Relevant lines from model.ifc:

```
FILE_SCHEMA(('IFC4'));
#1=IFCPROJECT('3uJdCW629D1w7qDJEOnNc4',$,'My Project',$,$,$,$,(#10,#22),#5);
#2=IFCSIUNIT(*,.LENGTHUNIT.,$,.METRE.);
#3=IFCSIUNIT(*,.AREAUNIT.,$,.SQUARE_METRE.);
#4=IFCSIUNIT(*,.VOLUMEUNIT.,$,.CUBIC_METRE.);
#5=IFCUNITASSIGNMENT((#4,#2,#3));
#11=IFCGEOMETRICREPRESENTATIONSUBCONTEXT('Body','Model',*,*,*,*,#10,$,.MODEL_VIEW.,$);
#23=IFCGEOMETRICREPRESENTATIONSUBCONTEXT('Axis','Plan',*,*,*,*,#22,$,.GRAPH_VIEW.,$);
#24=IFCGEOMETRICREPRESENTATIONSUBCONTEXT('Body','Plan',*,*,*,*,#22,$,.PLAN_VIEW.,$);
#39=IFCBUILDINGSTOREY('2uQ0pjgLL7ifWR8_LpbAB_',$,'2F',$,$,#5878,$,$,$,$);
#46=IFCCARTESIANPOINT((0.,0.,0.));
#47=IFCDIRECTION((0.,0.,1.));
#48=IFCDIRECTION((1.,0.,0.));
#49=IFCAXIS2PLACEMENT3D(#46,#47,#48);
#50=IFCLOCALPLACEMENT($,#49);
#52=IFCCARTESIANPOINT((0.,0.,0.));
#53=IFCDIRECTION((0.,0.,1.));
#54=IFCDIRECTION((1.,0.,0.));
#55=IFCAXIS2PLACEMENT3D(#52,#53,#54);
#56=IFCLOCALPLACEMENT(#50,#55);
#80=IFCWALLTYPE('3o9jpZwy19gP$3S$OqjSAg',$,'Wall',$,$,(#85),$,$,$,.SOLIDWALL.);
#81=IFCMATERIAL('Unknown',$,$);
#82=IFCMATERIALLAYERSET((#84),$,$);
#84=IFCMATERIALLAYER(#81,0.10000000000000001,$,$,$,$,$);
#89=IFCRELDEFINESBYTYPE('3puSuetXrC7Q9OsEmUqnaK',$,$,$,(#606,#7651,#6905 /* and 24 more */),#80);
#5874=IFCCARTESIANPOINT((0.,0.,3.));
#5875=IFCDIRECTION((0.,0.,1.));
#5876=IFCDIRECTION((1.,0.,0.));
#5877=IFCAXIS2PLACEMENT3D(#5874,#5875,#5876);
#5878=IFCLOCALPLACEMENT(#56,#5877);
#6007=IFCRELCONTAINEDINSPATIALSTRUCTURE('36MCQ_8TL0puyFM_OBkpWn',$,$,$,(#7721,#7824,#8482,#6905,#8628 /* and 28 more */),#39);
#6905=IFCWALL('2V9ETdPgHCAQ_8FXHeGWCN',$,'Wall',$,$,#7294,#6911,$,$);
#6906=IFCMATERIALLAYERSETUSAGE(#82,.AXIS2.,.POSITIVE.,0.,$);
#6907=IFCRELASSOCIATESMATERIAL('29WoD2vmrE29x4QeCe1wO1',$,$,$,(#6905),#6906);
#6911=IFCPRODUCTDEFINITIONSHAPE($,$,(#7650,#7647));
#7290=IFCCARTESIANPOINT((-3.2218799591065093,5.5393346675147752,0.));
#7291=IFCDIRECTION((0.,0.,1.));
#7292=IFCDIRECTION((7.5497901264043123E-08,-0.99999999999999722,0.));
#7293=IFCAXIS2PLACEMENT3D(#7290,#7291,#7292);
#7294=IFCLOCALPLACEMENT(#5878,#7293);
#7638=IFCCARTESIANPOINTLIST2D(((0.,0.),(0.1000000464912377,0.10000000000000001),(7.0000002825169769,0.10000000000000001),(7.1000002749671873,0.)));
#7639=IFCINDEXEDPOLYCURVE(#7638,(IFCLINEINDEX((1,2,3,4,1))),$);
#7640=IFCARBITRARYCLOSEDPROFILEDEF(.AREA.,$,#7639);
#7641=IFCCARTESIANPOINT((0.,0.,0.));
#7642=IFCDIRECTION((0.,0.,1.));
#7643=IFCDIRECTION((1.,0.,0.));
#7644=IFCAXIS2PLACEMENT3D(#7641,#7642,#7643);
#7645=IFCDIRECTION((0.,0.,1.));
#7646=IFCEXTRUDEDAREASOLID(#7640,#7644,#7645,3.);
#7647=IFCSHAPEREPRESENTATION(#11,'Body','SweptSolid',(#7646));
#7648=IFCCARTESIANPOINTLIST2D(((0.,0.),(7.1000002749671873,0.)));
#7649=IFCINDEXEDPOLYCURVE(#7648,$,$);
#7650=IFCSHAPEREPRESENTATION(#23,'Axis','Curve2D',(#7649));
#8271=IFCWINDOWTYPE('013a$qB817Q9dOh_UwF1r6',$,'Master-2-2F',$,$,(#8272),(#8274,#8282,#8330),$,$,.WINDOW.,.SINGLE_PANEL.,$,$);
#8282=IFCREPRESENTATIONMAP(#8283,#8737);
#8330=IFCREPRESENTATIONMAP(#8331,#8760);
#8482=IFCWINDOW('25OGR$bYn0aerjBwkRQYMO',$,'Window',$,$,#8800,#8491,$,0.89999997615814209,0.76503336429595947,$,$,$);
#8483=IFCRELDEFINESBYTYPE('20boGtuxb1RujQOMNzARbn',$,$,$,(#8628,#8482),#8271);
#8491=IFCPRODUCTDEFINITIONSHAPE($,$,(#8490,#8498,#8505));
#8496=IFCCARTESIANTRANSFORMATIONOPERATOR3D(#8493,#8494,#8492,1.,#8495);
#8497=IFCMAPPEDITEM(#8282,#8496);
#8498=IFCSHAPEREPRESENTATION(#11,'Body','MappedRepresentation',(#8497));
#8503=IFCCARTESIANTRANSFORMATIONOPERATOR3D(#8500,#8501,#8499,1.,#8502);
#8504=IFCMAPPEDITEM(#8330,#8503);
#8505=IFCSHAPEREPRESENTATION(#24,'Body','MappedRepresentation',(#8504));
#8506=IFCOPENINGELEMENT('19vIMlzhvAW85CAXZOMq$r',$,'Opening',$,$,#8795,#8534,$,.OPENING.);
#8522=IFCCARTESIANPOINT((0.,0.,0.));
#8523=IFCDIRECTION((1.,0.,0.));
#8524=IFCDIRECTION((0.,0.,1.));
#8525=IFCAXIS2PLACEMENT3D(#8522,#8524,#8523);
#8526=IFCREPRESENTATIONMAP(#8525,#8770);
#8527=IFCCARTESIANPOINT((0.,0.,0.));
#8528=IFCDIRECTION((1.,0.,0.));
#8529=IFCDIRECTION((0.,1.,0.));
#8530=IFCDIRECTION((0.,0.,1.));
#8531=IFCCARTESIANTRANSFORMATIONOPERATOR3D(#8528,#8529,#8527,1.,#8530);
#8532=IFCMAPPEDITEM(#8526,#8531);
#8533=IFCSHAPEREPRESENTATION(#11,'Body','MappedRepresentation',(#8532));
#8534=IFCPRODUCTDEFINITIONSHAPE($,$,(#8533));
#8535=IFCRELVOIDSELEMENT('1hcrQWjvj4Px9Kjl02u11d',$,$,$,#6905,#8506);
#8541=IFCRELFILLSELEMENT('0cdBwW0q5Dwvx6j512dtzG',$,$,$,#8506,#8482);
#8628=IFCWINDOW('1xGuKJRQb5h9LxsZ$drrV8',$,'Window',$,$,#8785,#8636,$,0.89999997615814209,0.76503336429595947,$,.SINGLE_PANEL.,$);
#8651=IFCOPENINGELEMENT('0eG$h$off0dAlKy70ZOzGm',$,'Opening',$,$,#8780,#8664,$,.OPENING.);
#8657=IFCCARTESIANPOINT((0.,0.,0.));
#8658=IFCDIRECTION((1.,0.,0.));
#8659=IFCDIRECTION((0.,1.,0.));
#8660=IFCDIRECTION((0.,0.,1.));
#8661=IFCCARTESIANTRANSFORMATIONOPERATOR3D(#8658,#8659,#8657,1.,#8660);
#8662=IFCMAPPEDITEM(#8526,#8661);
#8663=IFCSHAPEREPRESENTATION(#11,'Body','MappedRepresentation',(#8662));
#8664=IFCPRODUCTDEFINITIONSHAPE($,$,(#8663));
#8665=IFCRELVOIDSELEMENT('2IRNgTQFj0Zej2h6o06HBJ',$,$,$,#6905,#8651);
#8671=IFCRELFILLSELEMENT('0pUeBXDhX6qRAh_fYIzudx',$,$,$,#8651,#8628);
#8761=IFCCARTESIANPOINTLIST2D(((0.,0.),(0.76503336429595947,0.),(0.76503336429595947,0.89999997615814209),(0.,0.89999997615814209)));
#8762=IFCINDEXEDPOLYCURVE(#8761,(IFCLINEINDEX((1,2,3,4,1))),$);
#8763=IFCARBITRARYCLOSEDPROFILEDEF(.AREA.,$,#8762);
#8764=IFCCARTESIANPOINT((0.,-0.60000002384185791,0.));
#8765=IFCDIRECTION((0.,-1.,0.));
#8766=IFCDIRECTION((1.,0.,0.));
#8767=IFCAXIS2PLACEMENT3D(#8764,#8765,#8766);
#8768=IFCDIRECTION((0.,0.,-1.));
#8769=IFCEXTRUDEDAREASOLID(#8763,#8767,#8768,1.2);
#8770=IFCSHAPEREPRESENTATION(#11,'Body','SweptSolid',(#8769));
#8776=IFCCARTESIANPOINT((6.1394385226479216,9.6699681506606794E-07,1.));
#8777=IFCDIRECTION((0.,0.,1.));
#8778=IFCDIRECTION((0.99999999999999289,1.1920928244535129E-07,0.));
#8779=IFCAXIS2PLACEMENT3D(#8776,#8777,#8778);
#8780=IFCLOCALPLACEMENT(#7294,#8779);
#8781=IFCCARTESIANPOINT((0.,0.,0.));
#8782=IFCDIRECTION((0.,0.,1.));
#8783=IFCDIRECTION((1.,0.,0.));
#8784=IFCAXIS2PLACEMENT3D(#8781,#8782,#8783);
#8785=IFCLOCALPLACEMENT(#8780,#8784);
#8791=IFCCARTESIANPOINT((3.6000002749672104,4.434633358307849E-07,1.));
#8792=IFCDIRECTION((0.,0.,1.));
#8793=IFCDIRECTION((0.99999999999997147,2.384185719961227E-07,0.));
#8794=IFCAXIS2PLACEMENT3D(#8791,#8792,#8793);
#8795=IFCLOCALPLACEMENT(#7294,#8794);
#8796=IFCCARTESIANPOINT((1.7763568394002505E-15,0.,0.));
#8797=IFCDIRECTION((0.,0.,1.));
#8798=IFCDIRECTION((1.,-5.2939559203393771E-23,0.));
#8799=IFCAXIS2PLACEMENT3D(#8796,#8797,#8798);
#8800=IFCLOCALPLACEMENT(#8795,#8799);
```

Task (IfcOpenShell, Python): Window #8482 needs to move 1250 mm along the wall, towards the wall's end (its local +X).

```python
import ifcopenshell
import ifcopenshell.api.geometry
import ifcopenshell.util.placement
import ifcopenshell.util.unit

model = ifcopenshell.open("model.ifc")
unit_scale = ifcopenshell.util.unit.calculate_unit_scale(model)

window = model.by_guid("25OGR$bYn0aerjBwkRQYMO")
opening = window.FillsVoids[0].RelatingOpeningElement
wall = opening.VoidsElements[0].RelatingBuildingElement

wall_matrix = ifcopenshell.util.placement.get_local_placement(wall.ObjectPlacement)
shift = wall_matrix[:3, 0] * 1.25 / unit_scale
before = ifcopenshell.util.placement.get_local_placement(window.ObjectPlacement)[:3, 3].copy()

# The window is placed relative to its opening, so it follows when the opening moves.
matrix = ifcopenshell.util.placement.get_local_placement(opening.ObjectPlacement)
matrix[:3, 3] += shift
ifcopenshell.api.geometry.edit_object_placement(
    model, product=opening, matrix=matrix, is_si=False, should_transform_children=True
)

after = ifcopenshell.util.placement.get_local_placement(window.ObjectPlacement)[:3, 3]
print("window moved by", (after - before).round(3) + 0.0)

model.write("model-out.ifc")
```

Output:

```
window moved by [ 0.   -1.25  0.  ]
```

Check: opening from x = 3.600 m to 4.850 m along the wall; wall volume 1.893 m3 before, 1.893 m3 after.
